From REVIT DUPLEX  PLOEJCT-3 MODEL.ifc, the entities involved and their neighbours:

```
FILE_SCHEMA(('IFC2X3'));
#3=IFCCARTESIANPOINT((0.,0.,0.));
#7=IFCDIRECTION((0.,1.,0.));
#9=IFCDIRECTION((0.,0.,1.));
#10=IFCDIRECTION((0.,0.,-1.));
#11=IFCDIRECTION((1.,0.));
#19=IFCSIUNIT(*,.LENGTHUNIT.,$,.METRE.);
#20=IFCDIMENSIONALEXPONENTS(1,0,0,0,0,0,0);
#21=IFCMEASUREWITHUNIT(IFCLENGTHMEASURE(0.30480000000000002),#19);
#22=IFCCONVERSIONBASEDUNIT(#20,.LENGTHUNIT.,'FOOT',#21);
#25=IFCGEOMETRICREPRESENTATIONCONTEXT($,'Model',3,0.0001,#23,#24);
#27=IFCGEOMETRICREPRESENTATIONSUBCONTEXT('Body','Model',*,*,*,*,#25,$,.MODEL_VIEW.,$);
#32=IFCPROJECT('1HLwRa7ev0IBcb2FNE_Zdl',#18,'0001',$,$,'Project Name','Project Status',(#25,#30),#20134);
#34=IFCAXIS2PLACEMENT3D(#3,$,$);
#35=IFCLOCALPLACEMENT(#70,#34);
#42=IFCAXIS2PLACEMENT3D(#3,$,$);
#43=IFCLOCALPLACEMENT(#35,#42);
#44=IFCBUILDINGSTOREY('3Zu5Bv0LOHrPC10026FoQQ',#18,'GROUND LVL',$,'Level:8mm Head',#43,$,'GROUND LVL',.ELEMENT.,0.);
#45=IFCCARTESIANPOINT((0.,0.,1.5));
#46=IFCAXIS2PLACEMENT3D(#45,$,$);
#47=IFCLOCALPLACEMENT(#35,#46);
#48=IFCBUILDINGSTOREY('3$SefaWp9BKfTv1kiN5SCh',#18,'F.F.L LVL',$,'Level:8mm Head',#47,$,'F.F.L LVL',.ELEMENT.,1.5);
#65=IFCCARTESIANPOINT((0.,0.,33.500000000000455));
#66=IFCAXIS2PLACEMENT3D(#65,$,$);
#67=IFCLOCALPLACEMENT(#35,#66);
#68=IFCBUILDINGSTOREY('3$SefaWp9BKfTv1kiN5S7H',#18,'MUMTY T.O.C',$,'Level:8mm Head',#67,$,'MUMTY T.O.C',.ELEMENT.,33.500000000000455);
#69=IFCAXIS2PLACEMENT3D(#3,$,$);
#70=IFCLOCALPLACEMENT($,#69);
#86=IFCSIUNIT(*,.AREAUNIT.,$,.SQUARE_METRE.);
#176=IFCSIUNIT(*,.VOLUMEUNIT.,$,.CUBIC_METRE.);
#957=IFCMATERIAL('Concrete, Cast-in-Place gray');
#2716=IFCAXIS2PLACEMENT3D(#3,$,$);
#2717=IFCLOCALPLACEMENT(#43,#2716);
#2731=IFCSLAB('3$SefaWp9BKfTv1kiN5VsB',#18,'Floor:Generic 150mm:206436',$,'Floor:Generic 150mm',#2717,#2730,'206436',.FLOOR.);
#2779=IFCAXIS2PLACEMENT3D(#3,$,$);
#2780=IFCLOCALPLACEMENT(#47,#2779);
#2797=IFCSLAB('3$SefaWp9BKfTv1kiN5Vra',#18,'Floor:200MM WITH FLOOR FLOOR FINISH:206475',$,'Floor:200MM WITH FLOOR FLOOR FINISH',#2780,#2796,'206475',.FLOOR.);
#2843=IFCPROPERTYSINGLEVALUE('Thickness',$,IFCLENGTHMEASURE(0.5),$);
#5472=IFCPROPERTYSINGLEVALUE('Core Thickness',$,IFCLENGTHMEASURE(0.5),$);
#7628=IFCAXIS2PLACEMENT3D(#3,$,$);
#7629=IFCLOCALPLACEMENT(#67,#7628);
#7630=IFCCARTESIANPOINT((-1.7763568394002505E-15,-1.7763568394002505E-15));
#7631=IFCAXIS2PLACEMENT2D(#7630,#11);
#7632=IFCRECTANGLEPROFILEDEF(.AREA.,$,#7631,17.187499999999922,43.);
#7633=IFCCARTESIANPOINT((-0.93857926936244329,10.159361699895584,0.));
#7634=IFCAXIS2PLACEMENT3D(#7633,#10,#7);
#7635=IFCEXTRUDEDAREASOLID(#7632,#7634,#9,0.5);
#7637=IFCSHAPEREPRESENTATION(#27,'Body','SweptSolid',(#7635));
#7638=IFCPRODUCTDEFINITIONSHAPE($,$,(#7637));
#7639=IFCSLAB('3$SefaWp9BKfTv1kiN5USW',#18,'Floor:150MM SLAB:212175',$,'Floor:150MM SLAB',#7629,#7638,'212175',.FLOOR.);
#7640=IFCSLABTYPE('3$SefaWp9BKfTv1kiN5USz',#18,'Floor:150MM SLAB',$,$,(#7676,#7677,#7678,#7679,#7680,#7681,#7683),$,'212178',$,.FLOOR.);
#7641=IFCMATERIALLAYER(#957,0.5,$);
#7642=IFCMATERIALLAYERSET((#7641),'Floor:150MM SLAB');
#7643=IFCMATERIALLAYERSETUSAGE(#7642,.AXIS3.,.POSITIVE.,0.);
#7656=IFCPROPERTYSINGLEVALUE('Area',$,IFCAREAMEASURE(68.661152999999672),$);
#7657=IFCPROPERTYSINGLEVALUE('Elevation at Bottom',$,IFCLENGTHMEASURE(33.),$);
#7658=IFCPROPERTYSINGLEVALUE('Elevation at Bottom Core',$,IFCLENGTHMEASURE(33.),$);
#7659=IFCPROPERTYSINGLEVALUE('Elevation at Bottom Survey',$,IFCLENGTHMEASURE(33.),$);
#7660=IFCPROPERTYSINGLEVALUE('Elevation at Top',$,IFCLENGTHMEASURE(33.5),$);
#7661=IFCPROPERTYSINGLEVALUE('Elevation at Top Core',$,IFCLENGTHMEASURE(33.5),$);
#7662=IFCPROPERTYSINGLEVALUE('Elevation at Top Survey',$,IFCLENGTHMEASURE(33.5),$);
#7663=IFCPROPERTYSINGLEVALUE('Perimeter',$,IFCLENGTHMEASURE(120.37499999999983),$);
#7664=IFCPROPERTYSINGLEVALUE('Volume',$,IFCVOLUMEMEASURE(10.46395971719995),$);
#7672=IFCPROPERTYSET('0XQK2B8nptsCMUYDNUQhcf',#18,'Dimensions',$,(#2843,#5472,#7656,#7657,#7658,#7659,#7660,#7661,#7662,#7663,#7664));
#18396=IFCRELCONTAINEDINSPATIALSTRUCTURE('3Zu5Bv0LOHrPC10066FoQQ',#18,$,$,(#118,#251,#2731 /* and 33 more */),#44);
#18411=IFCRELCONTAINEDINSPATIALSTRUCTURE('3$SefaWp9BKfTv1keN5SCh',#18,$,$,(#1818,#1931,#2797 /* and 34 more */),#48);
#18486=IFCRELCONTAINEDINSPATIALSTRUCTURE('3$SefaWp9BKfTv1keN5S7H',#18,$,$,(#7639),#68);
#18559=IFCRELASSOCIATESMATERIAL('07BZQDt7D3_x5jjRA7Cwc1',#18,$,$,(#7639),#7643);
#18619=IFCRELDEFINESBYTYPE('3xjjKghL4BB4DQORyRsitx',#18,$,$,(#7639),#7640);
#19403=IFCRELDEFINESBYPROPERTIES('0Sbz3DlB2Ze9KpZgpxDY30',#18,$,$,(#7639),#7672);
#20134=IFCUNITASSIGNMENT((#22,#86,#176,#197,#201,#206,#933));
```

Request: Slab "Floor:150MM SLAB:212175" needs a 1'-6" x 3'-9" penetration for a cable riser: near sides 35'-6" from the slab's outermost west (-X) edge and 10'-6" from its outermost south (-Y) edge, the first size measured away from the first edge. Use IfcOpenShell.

```python
import numpy as np
import ifcopenshell
import ifcopenshell.api.feature
import ifcopenshell.api.geometry
import ifcopenshell.api.pset
import ifcopenshell.api.root
import ifcopenshell.geom
import ifcopenshell.util.element
import ifcopenshell.util.placement
import ifcopenshell.util.representation
import ifcopenshell.util.shape
import ifcopenshell.util.unit

model = ifcopenshell.open("REVIT DUPLEX  PLOEJCT-3 MODEL.ifc")
unit_scale = ifcopenshell.util.unit.calculate_unit_scale(model)
area_scale = ifcopenshell.util.unit.calculate_unit_scale(model, "AREAUNIT")
volume_scale = ifcopenshell.util.unit.calculate_unit_scale(model, "VOLUMEUNIT")
settings = ifcopenshell.geom.settings()


def volume(element):
    """Net volume in cubic metres, openings subtracted."""
    shape = ifcopenshell.geom.create_shape(settings, element)
    return ifcopenshell.util.shape.get_volume(shape.geometry)


slab = model.by_guid("3$SefaWp9BKfTv1kiN5USW")
before = volume(slab)

# Extent in the slab's own axes, in metres. The edges named are its -X and -Y sides.
slab_shape = ifcopenshell.geom.create_shape(settings, slab)
vertices = ifcopenshell.util.shape.get_vertices(slab_shape.geometry)
x_min, y_min, bottom = vertices.min(axis=0)
top = vertices[:, 2].max()

opening = ifcopenshell.api.root.create_entity(model, ifc_class="IfcOpeningElement", name="Cable riser opening")
context = ifcopenshell.util.representation.get_context(model, "Model", "Body", "MODEL_VIEW")
width, depth = 0.4572, 1.143
outline = [(0.0, 0.0), (width, 0.0), (width, depth), (0.0, depth), (0.0, 0.0)]
# Overshoot both faces by 50 mm so the cut is clean.
shape = ifcopenshell.api.geometry.add_slab_representation(
    model, context=context, depth=top - bottom + 0.1, polyline=outline
)
ifcopenshell.api.geometry.assign_representation(model, product=opening, representation=shape)

matrix = ifcopenshell.util.placement.get_local_placement(slab.ObjectPlacement)
matrix[:, 3] = matrix @ np.append(np.array([x_min + 10.8204, y_min + 3.2004, bottom - 0.05]) / unit_scale, 1.0)
ifcopenshell.api.geometry.edit_object_placement(model, product=opening, matrix=matrix, is_si=False)
ifcopenshell.api.feature.add_feature(model, feature=opening, element=slab)

after = volume(slab)

# Update the slab's stored quantities.
pset = model.by_id(ifcopenshell.util.element.get_pset(slab, "Dimensions", should_inherit=False)["id"])
ifcopenshell.api.pset.edit_pset(model, pset=pset, properties={
    "Area": model.create_entity("IfcAreaMeasure", after / (top - bottom) / area_scale),
    "Volume": model.create_entity("IfcVolumeMeasure", after / volume_scale),
})

print(f"slab volume {before:.3f} -> {after:.3f} m3")

model.write("REVIT DUPLEX  PLOEJCT-3 MODEL_rev.ifc")
```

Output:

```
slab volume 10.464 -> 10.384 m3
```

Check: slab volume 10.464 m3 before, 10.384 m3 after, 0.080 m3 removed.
